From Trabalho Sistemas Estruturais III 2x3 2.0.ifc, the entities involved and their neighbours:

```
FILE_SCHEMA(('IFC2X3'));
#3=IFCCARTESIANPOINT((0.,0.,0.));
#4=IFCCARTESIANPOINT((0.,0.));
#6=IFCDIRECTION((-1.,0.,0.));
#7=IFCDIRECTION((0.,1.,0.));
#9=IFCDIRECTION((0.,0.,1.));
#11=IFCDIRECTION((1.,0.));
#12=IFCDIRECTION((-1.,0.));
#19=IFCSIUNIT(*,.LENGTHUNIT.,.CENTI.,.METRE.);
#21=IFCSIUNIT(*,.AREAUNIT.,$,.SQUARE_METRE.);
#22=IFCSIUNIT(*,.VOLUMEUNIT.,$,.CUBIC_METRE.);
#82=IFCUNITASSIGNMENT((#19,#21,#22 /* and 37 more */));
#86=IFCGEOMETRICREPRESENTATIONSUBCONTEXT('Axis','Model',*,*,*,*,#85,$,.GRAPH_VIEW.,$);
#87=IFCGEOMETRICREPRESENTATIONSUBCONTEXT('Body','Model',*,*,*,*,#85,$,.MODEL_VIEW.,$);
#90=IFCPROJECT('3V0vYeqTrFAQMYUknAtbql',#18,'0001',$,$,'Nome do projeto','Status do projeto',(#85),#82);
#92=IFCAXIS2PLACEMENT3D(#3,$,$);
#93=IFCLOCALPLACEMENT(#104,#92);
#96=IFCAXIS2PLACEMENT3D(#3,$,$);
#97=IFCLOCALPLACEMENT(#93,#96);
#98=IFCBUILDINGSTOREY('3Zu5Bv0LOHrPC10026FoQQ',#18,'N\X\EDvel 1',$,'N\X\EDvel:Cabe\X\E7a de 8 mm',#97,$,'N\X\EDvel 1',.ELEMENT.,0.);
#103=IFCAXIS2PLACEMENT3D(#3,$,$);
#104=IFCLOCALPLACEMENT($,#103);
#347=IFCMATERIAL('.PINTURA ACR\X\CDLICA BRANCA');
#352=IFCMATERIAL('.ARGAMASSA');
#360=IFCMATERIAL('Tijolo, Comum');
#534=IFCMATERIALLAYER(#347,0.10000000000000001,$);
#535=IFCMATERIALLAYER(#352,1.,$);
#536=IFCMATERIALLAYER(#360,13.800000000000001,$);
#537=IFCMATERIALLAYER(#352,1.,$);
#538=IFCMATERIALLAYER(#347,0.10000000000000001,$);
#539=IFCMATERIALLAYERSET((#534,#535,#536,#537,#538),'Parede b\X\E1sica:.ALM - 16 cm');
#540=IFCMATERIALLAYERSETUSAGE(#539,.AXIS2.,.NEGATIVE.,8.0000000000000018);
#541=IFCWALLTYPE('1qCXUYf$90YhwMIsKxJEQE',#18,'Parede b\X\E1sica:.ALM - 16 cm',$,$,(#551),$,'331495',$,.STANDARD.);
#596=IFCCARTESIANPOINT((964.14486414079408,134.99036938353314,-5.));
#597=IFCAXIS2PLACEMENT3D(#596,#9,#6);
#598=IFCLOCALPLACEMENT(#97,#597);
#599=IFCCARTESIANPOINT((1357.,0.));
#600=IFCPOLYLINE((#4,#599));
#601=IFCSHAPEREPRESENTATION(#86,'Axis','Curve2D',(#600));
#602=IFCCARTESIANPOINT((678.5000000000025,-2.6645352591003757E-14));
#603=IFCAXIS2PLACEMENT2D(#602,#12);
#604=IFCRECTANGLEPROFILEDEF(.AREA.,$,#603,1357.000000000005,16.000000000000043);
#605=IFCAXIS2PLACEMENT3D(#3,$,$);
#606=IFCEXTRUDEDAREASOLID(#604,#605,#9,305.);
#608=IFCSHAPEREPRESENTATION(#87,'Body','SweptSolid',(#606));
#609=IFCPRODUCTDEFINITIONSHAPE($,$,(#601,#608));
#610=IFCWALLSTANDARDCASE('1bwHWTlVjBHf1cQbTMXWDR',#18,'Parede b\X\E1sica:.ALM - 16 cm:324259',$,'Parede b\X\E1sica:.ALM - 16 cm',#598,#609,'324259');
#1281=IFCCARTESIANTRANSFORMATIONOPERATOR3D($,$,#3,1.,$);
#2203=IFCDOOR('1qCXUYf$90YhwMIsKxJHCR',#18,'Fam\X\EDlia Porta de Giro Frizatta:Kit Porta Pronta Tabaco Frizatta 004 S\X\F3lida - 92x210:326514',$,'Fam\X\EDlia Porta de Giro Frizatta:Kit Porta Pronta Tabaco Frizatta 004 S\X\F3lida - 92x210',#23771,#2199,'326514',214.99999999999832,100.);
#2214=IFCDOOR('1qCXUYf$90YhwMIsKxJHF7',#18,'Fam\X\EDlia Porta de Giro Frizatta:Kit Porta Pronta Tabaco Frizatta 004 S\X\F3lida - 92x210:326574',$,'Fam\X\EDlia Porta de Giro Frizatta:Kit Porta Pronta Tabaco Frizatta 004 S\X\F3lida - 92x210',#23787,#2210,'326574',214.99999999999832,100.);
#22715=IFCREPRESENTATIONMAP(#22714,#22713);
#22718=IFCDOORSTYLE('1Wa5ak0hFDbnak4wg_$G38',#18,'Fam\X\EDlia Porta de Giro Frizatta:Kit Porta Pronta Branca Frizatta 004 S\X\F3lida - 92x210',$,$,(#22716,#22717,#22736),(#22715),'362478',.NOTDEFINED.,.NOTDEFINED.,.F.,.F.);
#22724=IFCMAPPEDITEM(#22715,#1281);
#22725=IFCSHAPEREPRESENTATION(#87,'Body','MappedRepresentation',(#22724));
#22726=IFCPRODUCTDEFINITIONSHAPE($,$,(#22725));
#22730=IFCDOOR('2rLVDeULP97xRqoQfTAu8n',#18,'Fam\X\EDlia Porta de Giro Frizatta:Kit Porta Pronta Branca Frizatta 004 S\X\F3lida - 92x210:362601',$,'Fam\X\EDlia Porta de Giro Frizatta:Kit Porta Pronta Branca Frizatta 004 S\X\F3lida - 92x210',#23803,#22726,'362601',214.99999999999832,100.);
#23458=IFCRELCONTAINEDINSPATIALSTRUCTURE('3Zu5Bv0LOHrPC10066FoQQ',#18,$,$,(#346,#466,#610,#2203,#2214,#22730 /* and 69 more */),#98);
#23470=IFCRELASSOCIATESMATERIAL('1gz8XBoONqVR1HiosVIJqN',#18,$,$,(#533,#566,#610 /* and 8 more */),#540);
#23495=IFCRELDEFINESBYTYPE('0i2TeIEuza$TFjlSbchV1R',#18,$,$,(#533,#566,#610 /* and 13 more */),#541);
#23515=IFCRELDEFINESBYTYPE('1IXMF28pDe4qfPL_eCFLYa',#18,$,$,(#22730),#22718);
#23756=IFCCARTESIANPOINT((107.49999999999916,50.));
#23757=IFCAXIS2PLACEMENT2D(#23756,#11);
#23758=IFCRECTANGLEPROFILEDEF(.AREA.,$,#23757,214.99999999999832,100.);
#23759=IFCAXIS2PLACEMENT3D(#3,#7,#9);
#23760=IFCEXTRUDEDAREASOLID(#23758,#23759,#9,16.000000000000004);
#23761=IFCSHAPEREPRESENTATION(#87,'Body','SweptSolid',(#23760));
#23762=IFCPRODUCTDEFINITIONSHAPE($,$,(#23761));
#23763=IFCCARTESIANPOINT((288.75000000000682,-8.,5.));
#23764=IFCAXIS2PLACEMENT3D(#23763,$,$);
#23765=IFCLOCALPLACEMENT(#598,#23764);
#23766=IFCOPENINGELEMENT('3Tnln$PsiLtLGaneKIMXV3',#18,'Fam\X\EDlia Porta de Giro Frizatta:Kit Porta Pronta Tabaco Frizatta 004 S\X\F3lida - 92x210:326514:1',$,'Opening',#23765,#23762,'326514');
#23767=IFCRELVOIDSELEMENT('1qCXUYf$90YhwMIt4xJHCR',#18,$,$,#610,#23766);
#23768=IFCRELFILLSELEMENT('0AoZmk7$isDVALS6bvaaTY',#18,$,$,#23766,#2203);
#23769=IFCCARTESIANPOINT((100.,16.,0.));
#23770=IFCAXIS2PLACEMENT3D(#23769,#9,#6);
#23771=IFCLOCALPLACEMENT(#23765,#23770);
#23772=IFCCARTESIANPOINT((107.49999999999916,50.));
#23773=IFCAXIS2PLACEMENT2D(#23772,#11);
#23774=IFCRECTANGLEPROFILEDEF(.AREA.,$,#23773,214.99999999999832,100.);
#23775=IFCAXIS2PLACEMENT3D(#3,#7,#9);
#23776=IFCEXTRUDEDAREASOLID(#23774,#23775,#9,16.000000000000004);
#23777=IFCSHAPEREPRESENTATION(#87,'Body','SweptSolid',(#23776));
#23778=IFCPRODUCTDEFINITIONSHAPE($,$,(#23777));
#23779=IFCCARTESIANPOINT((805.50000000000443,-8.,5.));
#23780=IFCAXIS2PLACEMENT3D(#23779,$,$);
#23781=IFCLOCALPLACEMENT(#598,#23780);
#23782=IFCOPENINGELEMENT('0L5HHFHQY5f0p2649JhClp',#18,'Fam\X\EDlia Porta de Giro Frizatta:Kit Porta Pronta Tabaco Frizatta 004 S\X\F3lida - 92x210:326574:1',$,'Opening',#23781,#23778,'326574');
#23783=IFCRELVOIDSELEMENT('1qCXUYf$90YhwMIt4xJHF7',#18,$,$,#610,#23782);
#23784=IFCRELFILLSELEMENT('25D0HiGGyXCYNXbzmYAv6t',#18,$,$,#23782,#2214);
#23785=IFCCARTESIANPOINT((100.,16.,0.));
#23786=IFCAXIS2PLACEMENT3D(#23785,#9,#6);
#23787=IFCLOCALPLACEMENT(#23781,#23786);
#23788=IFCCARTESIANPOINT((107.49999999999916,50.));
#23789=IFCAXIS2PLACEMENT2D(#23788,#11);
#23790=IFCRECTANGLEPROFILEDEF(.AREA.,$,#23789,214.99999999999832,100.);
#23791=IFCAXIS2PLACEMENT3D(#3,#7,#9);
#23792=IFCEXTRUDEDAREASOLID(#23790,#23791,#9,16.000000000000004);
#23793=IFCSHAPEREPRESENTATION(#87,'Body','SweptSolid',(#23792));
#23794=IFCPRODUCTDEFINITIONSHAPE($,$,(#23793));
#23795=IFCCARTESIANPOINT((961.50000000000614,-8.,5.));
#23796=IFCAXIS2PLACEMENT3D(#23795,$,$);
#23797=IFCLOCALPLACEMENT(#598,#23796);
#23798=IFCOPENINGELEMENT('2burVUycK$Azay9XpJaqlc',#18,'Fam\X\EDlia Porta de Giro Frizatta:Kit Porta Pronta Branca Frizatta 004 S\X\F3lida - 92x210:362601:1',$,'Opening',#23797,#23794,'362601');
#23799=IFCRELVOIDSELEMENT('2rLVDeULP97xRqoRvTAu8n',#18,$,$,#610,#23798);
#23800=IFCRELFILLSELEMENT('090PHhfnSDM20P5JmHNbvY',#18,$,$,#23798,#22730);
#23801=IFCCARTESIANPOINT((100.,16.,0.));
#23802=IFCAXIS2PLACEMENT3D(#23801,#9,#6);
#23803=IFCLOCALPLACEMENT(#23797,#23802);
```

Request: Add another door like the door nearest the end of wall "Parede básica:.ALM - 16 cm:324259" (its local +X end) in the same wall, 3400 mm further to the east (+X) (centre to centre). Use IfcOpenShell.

```python
import ifcopenshell
import ifcopenshell.api.feature
import ifcopenshell.api.geometry
import ifcopenshell.api.root
import ifcopenshell.geom
import ifcopenshell.util.element
import ifcopenshell.util.placement
import ifcopenshell.util.shape
import ifcopenshell.util.unit

model = ifcopenshell.open("Trabalho Sistemas Estruturais III 2x3 2.0.ifc")
unit_scale = ifcopenshell.util.unit.calculate_unit_scale(model)
settings = ifcopenshell.geom.settings()


def volume(element):
    """Net volume in cubic metres, openings subtracted."""
    shape = ifcopenshell.geom.create_shape(settings, element)
    return ifcopenshell.util.shape.get_volume(shape.geometry)


def reuse_history(source, copy):
    """copy_class also copies each property set's owner history, people and application; keep the originals."""
    for rel in copy.IsDefinedBy:
        if rel.is_a("IfcRelDefinesByProperties") and (history := rel.RelatingPropertyDefinition.OwnerHistory):
            rel.RelatingPropertyDefinition.OwnerHistory = source.OwnerHistory
            ifcopenshell.util.element.remove_deep2(model, history)


door = model.by_id(22730)
opening = door.FillsVoids[0].RelatingOpeningElement
wall = opening.VoidsElements[0].RelatingBuildingElement
before = volume(wall)
shift = ifcopenshell.util.placement.get_local_placement(wall.ObjectPlacement)[:3, 0] * -3.4 / unit_scale

# copy_class copies the void relationship, type, container and properties, but no geometry.
new_opening = ifcopenshell.api.root.copy_class(model, product=opening)
new_opening.Representation = ifcopenshell.util.element.copy_deep(
    model, opening.Representation, exclude=["IfcGeometricRepresentationContext", "IfcRepresentationMap"]
)
new_opening.Name = "Família Porta de Giro Frizatta:Kit Porta Pronta Branca Frizatta 004 Sólida - 92x210"
new_opening.Tag = None
new_door = ifcopenshell.api.root.copy_class(model, product=door)
new_door.Representation = ifcopenshell.util.element.copy_deep(
    model, door.Representation, exclude=["IfcGeometricRepresentationContext", "IfcRepresentationMap"]
)
new_door.Name = "Família Porta de Giro Frizatta:Kit Porta Pronta Branca Frizatta 004 Sólida - 92x210"
new_door.Tag = None
reuse_history(door, new_door)
fills = ifcopenshell.api.feature.add_filling(model, opening=new_opening, element=new_door)
fills.OwnerHistory = new_door.OwnerHistory  # required in IFC2X3

for old, new in ((opening, new_opening), (door, new_door)):
    matrix = ifcopenshell.util.placement.get_local_placement(old.ObjectPlacement)
    matrix[:3, 3] += shift
    ifcopenshell.api.geometry.edit_object_placement(model, product=new, matrix=matrix, is_si=False)

after = volume(wall)

print(f"wall volume {before:.3f} -> {after:.3f} m3")

model.write("Trabalho Sistemas Estruturais III 2x3 2.0_rev.ifc")
```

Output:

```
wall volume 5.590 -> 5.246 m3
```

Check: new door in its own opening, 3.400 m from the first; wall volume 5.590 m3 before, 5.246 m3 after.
